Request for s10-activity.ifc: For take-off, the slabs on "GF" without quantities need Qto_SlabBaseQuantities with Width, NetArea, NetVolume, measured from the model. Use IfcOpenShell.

First a look at what the model holds.

```python
import ifcopenshell
import ifcopenshell.util.element
import ifcopenshell.util.unit

model = ifcopenshell.open("s10-activity.ifc")
print(model.schema)
for unit_type in ("LENGTHUNIT", "AREAUNIT", "VOLUMEUNIT"):
    print(unit_type, ifcopenshell.util.unit.calculate_unit_scale(model, unit_type))
storey = next(s for s in model.by_type("IfcBuildingStorey") if s.Name == "GF")
slabs = [e for e in ifcopenshell.util.element.get_decomposition(storey) if e.is_a("IfcSlab")]
for e in sorted(slabs, key=lambda e: e.id()):
    print(e.id(), e.is_a(), e.Name, list(ifcopenshell.util.element.get_psets(e, qtos_only=True)), sep=" | ")
```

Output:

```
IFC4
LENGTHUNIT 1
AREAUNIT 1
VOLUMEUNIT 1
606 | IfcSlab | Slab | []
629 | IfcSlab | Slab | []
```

```python
import ifcopenshell
import ifcopenshell.api.pset
import ifcopenshell.geom
import ifcopenshell.util.element
import ifcopenshell.util.shape
import ifcopenshell.util.unit

model = ifcopenshell.open("s10-activity.ifc")
unit_scale = ifcopenshell.util.unit.calculate_unit_scale(model)
area_scale = ifcopenshell.util.unit.calculate_unit_scale(model, "AREAUNIT")
volume_scale = ifcopenshell.util.unit.calculate_unit_scale(model, "VOLUMEUNIT")
settings = ifcopenshell.geom.settings()

storey = next(s for s in model.by_type("IfcBuildingStorey") if s.Name == "GF")
slabs = [e for e in ifcopenshell.util.element.get_decomposition(storey) if e.is_a("IfcSlab")]

for e in sorted(slabs, key=lambda e: e.id()):
    if ifcopenshell.util.element.get_psets(e, qtos_only=True, should_inherit=False):
        continue
    # Geometry comes back in metres, in the element's own axes.
    shape = ifcopenshell.geom.create_shape(settings, e)
    values = {
        "Width": ifcopenshell.util.shape.get_z(shape.geometry) / unit_scale,
        "NetArea": ifcopenshell.util.shape.get_footprint_area(shape.geometry) / area_scale,
        "NetVolume": ifcopenshell.util.shape.get_volume(shape.geometry) / volume_scale,
    }
    qto = ifcopenshell.api.pset.add_qto(model, product=e, name="Qto_SlabBaseQuantities")
    ifcopenshell.api.pset.edit_qto(model, qto=qto, properties=values)
    print(e.id(), {k: round(v, 3) for k, v in values.items()})

model.write("s10-activity_edited.ifc")
```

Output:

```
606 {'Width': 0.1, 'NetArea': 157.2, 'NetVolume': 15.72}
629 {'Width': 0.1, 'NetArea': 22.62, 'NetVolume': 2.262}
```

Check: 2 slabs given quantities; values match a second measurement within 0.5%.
